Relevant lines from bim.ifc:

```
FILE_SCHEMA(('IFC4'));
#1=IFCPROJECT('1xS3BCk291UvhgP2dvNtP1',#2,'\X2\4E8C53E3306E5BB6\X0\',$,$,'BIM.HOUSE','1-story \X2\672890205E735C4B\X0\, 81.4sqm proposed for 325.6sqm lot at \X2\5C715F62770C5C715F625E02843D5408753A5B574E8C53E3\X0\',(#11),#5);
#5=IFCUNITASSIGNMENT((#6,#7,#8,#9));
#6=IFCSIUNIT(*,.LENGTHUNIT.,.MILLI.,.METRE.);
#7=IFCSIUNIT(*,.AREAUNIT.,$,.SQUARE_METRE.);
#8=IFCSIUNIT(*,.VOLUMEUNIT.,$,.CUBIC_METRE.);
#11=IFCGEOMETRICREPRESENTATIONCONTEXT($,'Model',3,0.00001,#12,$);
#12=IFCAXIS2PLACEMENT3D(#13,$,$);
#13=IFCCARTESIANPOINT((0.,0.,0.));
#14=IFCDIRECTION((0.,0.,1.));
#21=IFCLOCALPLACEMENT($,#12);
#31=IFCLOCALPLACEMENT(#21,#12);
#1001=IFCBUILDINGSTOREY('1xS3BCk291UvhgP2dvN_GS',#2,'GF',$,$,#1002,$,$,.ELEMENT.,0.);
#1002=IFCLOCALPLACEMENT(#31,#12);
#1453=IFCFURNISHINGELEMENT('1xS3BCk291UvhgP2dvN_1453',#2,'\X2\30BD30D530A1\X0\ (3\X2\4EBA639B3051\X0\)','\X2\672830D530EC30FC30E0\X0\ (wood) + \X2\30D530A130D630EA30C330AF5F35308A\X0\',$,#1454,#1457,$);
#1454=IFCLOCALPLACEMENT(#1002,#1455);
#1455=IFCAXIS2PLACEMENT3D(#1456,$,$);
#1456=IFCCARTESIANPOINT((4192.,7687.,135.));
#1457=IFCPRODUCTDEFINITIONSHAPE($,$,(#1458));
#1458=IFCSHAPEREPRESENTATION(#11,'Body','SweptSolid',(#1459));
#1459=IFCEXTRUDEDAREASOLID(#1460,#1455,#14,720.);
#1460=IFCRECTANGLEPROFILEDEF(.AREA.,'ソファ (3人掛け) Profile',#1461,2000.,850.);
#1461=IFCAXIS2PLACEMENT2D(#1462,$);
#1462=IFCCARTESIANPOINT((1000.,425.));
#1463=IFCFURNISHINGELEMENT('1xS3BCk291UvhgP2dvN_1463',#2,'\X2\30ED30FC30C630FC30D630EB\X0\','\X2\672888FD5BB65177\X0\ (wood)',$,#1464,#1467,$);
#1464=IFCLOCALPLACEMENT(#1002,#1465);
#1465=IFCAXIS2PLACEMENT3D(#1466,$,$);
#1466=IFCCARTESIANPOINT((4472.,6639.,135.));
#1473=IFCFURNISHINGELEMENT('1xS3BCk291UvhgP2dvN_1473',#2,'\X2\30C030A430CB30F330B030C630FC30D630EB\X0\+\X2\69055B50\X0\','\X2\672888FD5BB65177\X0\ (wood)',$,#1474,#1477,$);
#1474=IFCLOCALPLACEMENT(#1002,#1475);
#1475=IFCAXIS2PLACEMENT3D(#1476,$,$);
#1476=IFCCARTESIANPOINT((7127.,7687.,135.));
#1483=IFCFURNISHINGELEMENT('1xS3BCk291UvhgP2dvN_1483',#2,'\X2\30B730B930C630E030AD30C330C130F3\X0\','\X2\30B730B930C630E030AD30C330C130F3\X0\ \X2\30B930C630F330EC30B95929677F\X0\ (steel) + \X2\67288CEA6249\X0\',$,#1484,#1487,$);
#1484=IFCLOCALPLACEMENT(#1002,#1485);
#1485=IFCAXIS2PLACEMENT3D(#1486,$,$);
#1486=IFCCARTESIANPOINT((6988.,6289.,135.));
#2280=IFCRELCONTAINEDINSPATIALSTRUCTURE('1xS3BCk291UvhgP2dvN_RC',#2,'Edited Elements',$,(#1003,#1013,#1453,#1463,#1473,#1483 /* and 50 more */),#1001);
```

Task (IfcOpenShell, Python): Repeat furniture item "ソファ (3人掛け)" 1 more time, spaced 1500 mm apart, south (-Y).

```python
import numpy as np
import ifcopenshell
import ifcopenshell.api.geometry
import ifcopenshell.api.root
import ifcopenshell.util.element
import ifcopenshell.util.placement

model = ifcopenshell.open("bim.ifc")


def reuse_history(source, copy):
    """copy_class also copies each property set's owner history, people and application; keep the originals."""
    for rel in copy.IsDefinedBy:
        if rel.is_a("IfcRelDefinesByProperties") and (history := rel.RelatingPropertyDefinition.OwnerHistory):
            rel.RelatingPropertyDefinition.OwnerHistory = source.OwnerHistory
            ifcopenshell.util.element.remove_deep2(model, history)


source = model.by_guid("1xS3BCk291UvhgP2dvN_1453")
base = ifcopenshell.util.placement.get_local_placement(source.ObjectPlacement)
step = np.array([0.0, -1.0, 0.0]) * 1500.0

for i in range(1, 2):
    copy = ifcopenshell.api.root.copy_class(model, product=source)
    copy.Representation = ifcopenshell.util.element.copy_deep(
        model, source.Representation, exclude=["IfcGeometricRepresentationContext", "IfcRepresentationMap"]
    )
    reuse_history(source, copy)
    matrix = base.copy()
    matrix[:3, 3] += i * step
    print("added at", matrix[:3, 3].round(3) + 0.0)
    ifcopenshell.api.geometry.edit_object_placement(model, product=copy, matrix=matrix, is_si=False)

model.write("bim_updated.ifc")
```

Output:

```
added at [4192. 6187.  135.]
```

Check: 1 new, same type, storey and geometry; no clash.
